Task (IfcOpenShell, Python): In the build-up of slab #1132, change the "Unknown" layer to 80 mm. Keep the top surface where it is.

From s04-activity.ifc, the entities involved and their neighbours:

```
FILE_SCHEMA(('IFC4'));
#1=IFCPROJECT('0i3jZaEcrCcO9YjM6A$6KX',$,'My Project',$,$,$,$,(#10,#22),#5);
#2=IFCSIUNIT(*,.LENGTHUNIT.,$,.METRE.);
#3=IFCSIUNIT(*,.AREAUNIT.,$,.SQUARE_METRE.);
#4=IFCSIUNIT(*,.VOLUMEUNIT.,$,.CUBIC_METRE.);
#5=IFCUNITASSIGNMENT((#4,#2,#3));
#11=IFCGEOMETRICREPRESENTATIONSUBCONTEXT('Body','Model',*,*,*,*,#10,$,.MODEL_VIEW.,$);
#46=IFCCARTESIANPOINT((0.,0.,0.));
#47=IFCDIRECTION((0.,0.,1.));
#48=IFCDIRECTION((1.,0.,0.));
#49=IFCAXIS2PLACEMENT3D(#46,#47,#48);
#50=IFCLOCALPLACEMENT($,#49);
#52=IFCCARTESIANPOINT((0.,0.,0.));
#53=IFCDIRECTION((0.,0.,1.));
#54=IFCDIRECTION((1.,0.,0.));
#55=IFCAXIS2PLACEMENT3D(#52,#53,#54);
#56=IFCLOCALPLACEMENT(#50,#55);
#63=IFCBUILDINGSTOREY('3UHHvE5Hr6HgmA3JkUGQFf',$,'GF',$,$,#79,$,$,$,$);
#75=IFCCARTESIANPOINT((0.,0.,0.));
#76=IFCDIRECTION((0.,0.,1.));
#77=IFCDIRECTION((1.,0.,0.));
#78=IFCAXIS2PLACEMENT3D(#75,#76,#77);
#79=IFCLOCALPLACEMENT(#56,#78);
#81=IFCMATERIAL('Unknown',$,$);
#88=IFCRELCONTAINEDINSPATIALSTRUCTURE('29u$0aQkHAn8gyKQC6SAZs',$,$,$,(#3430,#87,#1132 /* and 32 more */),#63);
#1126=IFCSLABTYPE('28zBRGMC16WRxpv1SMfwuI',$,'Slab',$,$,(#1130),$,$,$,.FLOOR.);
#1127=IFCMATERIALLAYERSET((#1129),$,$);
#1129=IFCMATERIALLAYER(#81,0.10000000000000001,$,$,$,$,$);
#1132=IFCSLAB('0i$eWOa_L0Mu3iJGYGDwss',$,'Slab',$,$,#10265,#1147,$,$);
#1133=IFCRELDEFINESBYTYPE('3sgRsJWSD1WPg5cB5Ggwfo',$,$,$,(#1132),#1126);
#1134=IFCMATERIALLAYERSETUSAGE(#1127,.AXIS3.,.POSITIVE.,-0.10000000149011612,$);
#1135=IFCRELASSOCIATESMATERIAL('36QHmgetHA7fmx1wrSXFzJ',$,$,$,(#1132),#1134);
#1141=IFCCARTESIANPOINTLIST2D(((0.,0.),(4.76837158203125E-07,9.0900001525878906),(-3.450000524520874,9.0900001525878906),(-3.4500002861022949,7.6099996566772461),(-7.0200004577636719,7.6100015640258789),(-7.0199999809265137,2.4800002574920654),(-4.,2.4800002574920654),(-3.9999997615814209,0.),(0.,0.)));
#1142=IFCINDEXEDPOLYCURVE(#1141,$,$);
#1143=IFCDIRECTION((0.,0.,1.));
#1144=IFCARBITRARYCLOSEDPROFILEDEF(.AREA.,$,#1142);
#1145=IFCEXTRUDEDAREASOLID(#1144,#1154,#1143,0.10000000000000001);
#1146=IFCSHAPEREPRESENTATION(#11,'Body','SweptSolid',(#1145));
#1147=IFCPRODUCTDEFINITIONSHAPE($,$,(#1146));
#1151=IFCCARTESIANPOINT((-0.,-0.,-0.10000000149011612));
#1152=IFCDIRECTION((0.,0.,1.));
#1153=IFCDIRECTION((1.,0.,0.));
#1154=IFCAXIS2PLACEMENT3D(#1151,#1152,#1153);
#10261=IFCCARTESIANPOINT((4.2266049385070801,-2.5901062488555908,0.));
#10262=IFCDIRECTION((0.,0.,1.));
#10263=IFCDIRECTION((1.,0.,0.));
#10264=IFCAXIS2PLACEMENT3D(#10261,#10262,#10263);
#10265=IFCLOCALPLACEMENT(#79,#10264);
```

```python
import ifcopenshell
import ifcopenshell.util.element
import ifcopenshell.util.representation

model = ifcopenshell.open("s04-activity.ifc")

layer_set = model.by_id(1127)
layer = next(l for l in layer_set.MaterialLayers if l.Material and l.Material.Name == "Unknown")
change = 0.08 - layer.LayerThickness
layer.LayerThickness += change

# Geometry does not follow the layer set by itself.
slabs = [e for e in ifcopenshell.util.element.get_elements_by_material(model, layer_set) if e.is_a("IfcSlab")]
for slab in sorted(slabs, key=lambda e: e.id()):
    body = ifcopenshell.util.representation.get_representation(slab, "Model", "Body")
    solid = body.Items[0]
    old_depth = solid.Depth
    solid.Depth += change
    # Extruded upwards: lower the start of the extrusion so the top stays.
    x, y, z = solid.Position.Location.Coordinates
    solid.Position.Location = model.createIfcCartesianPoint((x, y, z - change))
    print(slab.id(), f"{old_depth:g} -> {solid.Depth:g}")

# The layers are counted up from the underside, which has moved.
for usage in {ifcopenshell.util.element.get_material(slab) for slab in slabs}:
    usage.OffsetFromReferenceLine -= change

model.write("s04-activity-out.ifc")
```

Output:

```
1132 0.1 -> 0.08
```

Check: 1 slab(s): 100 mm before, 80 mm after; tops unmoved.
